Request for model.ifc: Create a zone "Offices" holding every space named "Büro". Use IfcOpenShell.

First a look at what the model holds.

```python
import ifcopenshell

model = ifcopenshell.open("model.ifc")
print(model.schema)
seen = {}
for space in model.by_type("IfcSpace"):
    seen[space.LongName] = seen.get(space.LongName, 0) + 1
for name, count in sorted(seen.items(), key=str):
    print(count, "x", name)
print("zones:", [z.Name for z in model.by_type("IfcZone")][:20])
```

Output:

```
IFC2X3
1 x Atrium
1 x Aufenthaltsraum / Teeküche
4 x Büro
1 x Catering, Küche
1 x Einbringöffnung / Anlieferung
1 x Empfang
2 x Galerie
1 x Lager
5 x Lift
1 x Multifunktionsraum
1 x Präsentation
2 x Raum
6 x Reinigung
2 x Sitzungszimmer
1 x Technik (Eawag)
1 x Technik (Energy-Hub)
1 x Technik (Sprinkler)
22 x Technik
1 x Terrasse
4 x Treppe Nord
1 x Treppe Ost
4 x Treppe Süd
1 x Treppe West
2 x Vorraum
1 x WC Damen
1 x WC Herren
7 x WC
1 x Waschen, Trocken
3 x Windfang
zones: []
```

```python
import ifcopenshell
import ifcopenshell.api.group
import ifcopenshell.api.root

model = ifcopenshell.open("model.ifc")

names = {"Büro"}
spaces = [s for s in model.by_type("IfcSpace") if s.LongName in names]

zone = ifcopenshell.api.root.create_entity(model, ifc_class="IfcZone", name="Offices")
ifcopenshell.api.group.assign_group(model, products=spaces, group=zone)
print(len(spaces), "spaces in", zone.Name)

model.write("model-out.ifc")
```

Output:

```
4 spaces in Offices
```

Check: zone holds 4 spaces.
